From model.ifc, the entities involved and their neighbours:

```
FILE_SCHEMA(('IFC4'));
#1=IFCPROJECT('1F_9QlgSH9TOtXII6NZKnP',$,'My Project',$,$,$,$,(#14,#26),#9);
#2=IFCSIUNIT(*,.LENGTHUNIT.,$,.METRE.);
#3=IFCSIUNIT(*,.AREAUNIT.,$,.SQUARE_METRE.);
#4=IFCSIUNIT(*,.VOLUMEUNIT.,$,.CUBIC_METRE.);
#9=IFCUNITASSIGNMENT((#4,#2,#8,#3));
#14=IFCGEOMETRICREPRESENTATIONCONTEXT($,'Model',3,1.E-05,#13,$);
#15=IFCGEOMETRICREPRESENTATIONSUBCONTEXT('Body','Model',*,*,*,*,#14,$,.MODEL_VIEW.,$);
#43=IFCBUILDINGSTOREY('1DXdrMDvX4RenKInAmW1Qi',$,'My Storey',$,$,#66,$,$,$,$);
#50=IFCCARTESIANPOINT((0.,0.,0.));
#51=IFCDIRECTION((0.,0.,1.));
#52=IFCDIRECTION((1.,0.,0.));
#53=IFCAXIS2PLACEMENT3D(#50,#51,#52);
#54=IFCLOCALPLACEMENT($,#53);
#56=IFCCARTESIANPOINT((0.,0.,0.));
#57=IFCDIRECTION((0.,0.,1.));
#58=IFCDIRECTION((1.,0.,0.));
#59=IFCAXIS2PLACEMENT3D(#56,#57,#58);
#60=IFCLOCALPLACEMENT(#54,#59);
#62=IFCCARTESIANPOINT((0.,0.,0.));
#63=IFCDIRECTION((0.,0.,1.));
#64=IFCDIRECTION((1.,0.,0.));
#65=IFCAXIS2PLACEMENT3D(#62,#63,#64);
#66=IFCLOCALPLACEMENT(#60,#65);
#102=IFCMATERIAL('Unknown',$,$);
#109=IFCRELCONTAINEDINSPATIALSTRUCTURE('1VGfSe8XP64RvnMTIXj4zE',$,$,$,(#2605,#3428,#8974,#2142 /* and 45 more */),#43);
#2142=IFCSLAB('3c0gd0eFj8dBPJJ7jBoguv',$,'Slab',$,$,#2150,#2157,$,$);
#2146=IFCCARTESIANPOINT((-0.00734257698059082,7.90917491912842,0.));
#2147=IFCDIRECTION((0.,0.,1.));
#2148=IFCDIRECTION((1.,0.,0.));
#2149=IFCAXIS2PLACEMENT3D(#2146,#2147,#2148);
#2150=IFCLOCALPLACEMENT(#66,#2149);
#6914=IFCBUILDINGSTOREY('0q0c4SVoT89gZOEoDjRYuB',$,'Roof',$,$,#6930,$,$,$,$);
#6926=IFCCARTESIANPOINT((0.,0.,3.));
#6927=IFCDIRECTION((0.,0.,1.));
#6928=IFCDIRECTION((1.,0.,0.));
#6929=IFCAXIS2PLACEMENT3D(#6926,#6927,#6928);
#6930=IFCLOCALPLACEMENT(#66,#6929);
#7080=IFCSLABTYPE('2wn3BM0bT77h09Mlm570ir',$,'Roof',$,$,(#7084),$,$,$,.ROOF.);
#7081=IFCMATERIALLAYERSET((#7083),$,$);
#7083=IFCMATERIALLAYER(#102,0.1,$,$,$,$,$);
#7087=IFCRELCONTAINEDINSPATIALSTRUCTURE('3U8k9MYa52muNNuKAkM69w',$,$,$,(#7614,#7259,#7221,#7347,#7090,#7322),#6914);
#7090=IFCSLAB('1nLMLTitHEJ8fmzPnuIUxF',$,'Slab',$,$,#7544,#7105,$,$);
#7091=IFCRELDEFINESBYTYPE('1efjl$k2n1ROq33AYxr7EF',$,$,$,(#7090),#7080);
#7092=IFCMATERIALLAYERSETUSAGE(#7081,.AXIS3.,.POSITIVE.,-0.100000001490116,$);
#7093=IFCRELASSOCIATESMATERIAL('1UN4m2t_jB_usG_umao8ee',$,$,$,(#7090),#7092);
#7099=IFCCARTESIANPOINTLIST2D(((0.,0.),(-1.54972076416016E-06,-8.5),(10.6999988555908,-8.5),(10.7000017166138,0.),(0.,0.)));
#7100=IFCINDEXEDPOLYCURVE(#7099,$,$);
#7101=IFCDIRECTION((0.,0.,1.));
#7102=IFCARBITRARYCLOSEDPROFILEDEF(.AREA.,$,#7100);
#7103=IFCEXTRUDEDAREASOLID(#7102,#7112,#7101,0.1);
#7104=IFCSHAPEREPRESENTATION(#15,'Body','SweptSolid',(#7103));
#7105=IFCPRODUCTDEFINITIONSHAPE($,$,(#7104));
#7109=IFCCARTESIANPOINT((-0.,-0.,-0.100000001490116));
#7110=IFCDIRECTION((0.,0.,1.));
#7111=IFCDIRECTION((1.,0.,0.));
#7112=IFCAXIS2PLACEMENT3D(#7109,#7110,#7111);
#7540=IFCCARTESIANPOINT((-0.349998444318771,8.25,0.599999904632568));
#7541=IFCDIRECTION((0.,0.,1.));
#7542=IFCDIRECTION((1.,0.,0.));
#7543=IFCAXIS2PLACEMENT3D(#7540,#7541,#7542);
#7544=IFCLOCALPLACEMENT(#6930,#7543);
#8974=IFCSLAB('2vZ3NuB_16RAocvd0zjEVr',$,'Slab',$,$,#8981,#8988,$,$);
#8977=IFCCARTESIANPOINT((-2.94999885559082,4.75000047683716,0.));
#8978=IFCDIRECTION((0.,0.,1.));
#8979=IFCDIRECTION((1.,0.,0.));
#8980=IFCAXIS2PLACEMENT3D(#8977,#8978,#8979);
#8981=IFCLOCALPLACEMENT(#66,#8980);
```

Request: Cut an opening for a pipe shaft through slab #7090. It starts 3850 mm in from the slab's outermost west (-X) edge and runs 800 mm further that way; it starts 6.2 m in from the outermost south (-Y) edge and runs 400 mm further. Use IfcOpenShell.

```python
import numpy as np
import ifcopenshell
import ifcopenshell.api.feature
import ifcopenshell.api.geometry
import ifcopenshell.api.root
import ifcopenshell.geom
import ifcopenshell.util.placement
import ifcopenshell.util.representation
import ifcopenshell.util.shape
import ifcopenshell.util.unit

model = ifcopenshell.open("model.ifc")
unit_scale = ifcopenshell.util.unit.calculate_unit_scale(model)
settings = ifcopenshell.geom.settings()


def volume(element):
    """Net volume in cubic metres, openings subtracted."""
    shape = ifcopenshell.geom.create_shape(settings, element)
    return ifcopenshell.util.shape.get_volume(shape.geometry)


slab = model.by_guid("1nLMLTitHEJ8fmzPnuIUxF")
before = volume(slab)

# Extent in the slab's own axes, in metres. The edges named are its -X and -Y sides.
slab_shape = ifcopenshell.geom.create_shape(settings, slab)
vertices = ifcopenshell.util.shape.get_vertices(slab_shape.geometry)
x_min, y_min, bottom = vertices.min(axis=0)
top = vertices[:, 2].max()

opening = ifcopenshell.api.root.create_entity(model, ifc_class="IfcOpeningElement", name="Pipe shaft opening", predefined_type="OPENING")
context = ifcopenshell.util.representation.get_context(model, "Model", "Body", "MODEL_VIEW")
width, depth = 0.8, 0.4
outline = [(0.0, 0.0), (width, 0.0), (width, depth), (0.0, depth), (0.0, 0.0)]
# Overshoot both faces by 50 mm so the cut is clean.
shape = ifcopenshell.api.geometry.add_slab_representation(
    model, context=context, depth=top - bottom + 0.1, polyline=outline
)
ifcopenshell.api.geometry.assign_representation(model, product=opening, representation=shape)

matrix = ifcopenshell.util.placement.get_local_placement(slab.ObjectPlacement)
matrix[:, 3] = matrix @ np.append(np.array([x_min + 3.85, y_min + 6.2, bottom - 0.05]) / unit_scale, 1.0)
ifcopenshell.api.geometry.edit_object_placement(model, product=opening, matrix=matrix, is_si=False)
ifcopenshell.api.feature.add_feature(model, feature=opening, element=slab)

after = volume(slab)

print(f"slab volume {before:.3f} -> {after:.3f} m3")

model.write("model_rev.ifc")
```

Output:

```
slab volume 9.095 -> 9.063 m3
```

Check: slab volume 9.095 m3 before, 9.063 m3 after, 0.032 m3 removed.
